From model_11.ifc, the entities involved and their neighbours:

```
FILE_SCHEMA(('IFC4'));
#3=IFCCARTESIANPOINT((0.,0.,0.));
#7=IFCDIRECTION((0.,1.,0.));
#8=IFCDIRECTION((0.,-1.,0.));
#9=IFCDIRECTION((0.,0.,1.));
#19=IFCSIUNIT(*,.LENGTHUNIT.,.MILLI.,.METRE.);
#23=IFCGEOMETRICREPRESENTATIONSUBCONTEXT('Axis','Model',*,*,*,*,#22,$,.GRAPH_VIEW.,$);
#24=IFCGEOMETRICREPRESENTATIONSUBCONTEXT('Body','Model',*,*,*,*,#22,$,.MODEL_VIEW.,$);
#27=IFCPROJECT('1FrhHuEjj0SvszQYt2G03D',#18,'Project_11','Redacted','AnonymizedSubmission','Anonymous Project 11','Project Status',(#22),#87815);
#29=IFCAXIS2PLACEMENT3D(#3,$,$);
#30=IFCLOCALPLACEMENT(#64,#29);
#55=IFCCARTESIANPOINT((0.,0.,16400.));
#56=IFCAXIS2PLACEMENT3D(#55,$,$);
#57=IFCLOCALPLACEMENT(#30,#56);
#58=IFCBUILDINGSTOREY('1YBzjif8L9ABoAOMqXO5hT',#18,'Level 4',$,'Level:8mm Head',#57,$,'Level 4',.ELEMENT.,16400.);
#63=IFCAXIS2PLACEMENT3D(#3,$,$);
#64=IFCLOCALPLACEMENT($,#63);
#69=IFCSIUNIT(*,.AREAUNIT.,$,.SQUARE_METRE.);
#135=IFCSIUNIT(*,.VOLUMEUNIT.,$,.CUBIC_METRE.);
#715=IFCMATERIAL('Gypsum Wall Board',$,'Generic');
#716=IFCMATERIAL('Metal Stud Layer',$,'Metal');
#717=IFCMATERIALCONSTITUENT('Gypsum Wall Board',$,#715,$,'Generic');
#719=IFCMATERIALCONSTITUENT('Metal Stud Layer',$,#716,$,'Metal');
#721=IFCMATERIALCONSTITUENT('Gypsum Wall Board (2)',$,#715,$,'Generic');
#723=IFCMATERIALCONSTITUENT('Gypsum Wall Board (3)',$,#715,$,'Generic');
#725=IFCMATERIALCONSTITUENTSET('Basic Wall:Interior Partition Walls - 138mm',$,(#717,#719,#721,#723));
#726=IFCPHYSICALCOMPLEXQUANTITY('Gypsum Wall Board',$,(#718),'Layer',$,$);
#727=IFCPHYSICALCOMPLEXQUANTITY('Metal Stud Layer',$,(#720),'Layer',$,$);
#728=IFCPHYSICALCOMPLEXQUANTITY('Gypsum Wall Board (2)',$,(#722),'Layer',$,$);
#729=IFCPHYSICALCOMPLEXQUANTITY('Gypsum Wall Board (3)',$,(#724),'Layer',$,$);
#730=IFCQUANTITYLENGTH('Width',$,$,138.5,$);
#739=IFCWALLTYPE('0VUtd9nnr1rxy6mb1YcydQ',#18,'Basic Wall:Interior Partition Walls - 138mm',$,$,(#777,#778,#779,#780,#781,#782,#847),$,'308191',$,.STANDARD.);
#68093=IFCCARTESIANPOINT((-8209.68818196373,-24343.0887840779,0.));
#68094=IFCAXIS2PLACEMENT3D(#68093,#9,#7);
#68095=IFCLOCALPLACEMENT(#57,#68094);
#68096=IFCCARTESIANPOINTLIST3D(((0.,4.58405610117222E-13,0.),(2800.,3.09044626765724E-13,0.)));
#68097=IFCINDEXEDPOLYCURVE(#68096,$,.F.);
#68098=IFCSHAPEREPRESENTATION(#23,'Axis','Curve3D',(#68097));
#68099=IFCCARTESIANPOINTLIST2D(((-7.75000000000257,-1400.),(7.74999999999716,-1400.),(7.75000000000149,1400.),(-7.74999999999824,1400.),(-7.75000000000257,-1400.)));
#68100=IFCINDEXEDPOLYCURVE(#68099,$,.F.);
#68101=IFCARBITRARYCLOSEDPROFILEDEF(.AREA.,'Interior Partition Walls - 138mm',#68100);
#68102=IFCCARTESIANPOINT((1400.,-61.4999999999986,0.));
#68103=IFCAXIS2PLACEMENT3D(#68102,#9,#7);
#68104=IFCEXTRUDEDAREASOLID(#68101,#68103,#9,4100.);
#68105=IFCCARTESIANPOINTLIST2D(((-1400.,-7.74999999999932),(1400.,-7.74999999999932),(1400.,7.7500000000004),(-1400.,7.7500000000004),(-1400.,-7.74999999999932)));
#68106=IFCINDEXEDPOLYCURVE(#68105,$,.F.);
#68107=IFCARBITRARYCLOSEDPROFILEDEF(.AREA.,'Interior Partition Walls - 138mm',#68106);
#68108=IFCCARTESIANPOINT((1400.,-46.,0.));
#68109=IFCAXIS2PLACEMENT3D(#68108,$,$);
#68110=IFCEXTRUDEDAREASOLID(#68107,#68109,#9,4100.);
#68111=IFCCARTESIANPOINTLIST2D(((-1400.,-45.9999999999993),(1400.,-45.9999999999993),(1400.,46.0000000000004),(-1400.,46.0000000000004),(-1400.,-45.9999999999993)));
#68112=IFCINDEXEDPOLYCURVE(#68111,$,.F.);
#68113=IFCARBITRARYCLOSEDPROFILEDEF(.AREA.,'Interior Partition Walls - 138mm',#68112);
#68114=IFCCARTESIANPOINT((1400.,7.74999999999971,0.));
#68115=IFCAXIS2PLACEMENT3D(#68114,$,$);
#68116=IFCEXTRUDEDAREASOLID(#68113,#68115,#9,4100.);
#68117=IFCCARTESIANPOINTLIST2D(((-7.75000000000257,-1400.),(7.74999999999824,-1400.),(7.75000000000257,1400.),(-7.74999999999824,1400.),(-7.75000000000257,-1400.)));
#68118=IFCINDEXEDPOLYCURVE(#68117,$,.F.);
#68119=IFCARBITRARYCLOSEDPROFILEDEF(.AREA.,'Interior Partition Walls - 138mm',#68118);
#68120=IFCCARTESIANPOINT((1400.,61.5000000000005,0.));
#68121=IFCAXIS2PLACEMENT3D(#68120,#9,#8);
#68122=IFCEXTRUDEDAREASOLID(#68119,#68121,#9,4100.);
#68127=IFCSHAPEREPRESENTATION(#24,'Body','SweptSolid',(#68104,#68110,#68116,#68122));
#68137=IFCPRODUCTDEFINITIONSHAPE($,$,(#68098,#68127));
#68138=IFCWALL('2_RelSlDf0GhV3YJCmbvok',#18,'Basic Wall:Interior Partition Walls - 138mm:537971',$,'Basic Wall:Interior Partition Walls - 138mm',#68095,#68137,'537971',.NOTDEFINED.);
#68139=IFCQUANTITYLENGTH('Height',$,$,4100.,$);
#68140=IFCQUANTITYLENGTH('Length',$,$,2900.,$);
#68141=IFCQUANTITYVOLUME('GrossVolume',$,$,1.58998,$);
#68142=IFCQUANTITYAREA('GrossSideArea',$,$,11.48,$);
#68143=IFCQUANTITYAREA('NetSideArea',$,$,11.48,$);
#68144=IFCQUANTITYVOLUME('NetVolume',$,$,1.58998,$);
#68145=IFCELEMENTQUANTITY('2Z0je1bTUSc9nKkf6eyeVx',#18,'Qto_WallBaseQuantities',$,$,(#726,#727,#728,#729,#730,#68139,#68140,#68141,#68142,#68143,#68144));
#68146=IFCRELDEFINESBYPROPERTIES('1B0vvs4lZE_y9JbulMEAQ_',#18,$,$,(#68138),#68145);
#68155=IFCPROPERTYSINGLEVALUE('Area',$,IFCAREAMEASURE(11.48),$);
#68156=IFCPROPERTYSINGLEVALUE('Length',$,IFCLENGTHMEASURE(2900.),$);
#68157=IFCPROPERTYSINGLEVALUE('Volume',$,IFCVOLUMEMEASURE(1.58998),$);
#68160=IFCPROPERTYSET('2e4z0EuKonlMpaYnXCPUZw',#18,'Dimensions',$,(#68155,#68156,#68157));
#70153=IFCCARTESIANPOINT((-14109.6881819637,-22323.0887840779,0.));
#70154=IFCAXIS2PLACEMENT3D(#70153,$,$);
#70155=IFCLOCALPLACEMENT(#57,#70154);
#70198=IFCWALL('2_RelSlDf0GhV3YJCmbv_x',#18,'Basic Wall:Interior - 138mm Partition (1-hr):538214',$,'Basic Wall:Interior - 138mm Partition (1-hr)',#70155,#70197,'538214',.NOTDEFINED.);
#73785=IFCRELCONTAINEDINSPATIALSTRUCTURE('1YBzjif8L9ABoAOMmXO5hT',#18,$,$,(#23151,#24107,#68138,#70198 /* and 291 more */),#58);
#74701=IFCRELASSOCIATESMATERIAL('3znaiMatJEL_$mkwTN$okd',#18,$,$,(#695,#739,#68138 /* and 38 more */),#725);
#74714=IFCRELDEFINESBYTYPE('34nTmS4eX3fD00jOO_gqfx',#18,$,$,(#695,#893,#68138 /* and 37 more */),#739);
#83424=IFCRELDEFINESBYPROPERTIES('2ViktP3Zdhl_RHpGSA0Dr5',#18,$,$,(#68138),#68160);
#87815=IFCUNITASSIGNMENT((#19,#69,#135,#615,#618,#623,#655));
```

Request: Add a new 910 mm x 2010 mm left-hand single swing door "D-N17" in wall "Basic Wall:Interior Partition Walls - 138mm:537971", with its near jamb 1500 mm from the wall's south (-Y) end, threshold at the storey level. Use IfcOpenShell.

```python
import numpy as np
import ifcopenshell
import ifcopenshell.api.feature
import ifcopenshell.api.geometry
import ifcopenshell.api.pset
import ifcopenshell.api.root
import ifcopenshell.api.spatial
import ifcopenshell.geom
import ifcopenshell.util.element
import ifcopenshell.util.placement
import ifcopenshell.util.representation
import ifcopenshell.util.shape
import ifcopenshell.util.unit

model = ifcopenshell.open("model_11.ifc")
unit_scale = ifcopenshell.util.unit.calculate_unit_scale(model)
area_scale = ifcopenshell.util.unit.calculate_unit_scale(model, "AREAUNIT")
volume_scale = ifcopenshell.util.unit.calculate_unit_scale(model, "VOLUMEUNIT")
settings = ifcopenshell.geom.settings()


def volume(element):
    """Net volume in cubic metres, openings subtracted."""
    shape = ifcopenshell.geom.create_shape(settings, element)
    return ifcopenshell.util.shape.get_volume(shape.geometry)


wall = model.by_guid("2_RelSlDf0GhV3YJCmbvok")
storey = ifcopenshell.util.element.get_container(wall, ifc_class="IfcBuildingStorey")
context = ifcopenshell.util.representation.get_context(model, "Model", "Body", "MODEL_VIEW")
before = volume(wall)

width, height, from_end, sill = 0.91, 2.01, 1.5, 0.0  # metres

# The wall runs along its own X axis, and the end named is its -X end.
wall_shape = ifcopenshell.geom.create_shape(settings, wall)
x, y, z = ifcopenshell.util.shape.get_vertices(wall_shape.geometry).T
start = x.min() + from_end
face, thickness = float(y.min()), float(y.max() - y.min())
wall_matrix = ifcopenshell.util.placement.get_local_placement(wall.ObjectPlacement)
level = ifcopenshell.util.placement.get_local_placement(storey.ObjectPlacement)[2, 3]


def in_wall(x, y):
    """Placement at x, y metres in the wall's axes, at sill height."""
    matrix = wall_matrix.copy()
    matrix[:, 3] = wall_matrix @ np.array([x / unit_scale, y / unit_scale, 0.0, 1.0])
    matrix[2, 3] = level + sill / unit_scale
    return matrix


# Opening: a box that overshoots both wall faces by 50 mm.
opening = ifcopenshell.api.root.create_entity(model, ifc_class="IfcOpeningElement", predefined_type="OPENING")
box = ifcopenshell.api.geometry.add_wall_representation(
    model, context=context, length=width, height=height, thickness=thickness + 0.1
)
ifcopenshell.api.geometry.assign_representation(model, product=opening, representation=box)
ifcopenshell.api.geometry.edit_object_placement(model, product=opening, matrix=in_wall(start, face - 0.05), is_si=False)
ifcopenshell.api.feature.add_feature(model, feature=opening, element=wall)

door = ifcopenshell.api.root.create_entity(model, ifc_class="IfcDoor", name="D-N17", predefined_type="DOOR")
door.OverallWidth, door.OverallHeight = width / unit_scale, height / unit_scale
door.OperationType = "SINGLE_SWING_LEFT"
body = ifcopenshell.api.geometry.add_door_representation(
    model,
    context=context,
    overall_width=door.OverallWidth,
    overall_height=door.OverallHeight,
    operation_type="SINGLE_SWING_LEFT",
    lining_properties={"LiningDepth": thickness / unit_scale, "ThresholdDepth": thickness / unit_scale},
)
ifcopenshell.api.geometry.assign_representation(model, product=door, representation=body)
ifcopenshell.api.spatial.assign_container(model, products=[door], relating_structure=storey)
ifcopenshell.api.feature.add_filling(model, opening=opening, element=door)

# The lining spans the wall, so the door starts at the wall face.
ifcopenshell.api.geometry.edit_object_placement(model, product=door, matrix=in_wall(start, face), is_si=False)

after = volume(wall)

# Update the wall's stored quantities.
qto = model.by_id(ifcopenshell.util.element.get_pset(wall, "Qto_WallBaseQuantities", should_inherit=False)["id"])
ifcopenshell.api.pset.edit_qto(model, qto=qto, properties={
    "NetSideArea": after / thickness / area_scale,
    "NetVolume": after / volume_scale,
})
pset = model.by_id(ifcopenshell.util.element.get_pset(wall, "Dimensions", should_inherit=False)["id"])
ifcopenshell.api.pset.edit_pset(model, pset=pset, properties={
    "Area": model.create_entity("IfcAreaMeasure", after / thickness / area_scale),
    "Volume": model.create_entity("IfcVolumeMeasure", after / volume_scale),
})

print(f"wall volume {before:.3f} -> {after:.3f} m3")

model.write("model_11-out.ifc")
```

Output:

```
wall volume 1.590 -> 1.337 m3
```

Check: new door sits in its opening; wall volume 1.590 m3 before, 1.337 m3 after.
